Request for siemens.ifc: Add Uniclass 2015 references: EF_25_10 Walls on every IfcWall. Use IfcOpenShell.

First a look at what the model holds.

```python
import ifcopenshell

model = ifcopenshell.open("siemens.ifc")
print(model.schema)
print("classifications:", [c.Name for c in model.by_type("IfcClassification")])
for ifc_class in ("IfcDoor", "IfcRoof", "IfcStair", "IfcWall", "IfcWindow"):
    print(ifc_class, len(model.by_type(ifc_class)))
```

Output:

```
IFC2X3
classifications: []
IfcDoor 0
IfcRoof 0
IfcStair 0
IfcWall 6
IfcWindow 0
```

```python
import ifcopenshell
import ifcopenshell.api.classification

model = ifcopenshell.open("siemens.ifc")

# IFC2X3 requires Source and Edition and has no link from the project to the system.
system = model.create_entity("IfcClassification", Source="NBS", Edition="2015", Name="Uniclass 2015")

codes = {
    "IfcWall": ("EF_25_10", "Walls"),
}
for ifc_class, (code, name) in codes.items():
    products = model.by_type(ifc_class)
    ifcopenshell.api.classification.add_reference(
        model, products=products, classification=system, identification=code, name=name
    )
    print(code, len(products))

model.write("siemens-out.ifc")
```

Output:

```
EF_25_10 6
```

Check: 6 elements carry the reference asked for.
